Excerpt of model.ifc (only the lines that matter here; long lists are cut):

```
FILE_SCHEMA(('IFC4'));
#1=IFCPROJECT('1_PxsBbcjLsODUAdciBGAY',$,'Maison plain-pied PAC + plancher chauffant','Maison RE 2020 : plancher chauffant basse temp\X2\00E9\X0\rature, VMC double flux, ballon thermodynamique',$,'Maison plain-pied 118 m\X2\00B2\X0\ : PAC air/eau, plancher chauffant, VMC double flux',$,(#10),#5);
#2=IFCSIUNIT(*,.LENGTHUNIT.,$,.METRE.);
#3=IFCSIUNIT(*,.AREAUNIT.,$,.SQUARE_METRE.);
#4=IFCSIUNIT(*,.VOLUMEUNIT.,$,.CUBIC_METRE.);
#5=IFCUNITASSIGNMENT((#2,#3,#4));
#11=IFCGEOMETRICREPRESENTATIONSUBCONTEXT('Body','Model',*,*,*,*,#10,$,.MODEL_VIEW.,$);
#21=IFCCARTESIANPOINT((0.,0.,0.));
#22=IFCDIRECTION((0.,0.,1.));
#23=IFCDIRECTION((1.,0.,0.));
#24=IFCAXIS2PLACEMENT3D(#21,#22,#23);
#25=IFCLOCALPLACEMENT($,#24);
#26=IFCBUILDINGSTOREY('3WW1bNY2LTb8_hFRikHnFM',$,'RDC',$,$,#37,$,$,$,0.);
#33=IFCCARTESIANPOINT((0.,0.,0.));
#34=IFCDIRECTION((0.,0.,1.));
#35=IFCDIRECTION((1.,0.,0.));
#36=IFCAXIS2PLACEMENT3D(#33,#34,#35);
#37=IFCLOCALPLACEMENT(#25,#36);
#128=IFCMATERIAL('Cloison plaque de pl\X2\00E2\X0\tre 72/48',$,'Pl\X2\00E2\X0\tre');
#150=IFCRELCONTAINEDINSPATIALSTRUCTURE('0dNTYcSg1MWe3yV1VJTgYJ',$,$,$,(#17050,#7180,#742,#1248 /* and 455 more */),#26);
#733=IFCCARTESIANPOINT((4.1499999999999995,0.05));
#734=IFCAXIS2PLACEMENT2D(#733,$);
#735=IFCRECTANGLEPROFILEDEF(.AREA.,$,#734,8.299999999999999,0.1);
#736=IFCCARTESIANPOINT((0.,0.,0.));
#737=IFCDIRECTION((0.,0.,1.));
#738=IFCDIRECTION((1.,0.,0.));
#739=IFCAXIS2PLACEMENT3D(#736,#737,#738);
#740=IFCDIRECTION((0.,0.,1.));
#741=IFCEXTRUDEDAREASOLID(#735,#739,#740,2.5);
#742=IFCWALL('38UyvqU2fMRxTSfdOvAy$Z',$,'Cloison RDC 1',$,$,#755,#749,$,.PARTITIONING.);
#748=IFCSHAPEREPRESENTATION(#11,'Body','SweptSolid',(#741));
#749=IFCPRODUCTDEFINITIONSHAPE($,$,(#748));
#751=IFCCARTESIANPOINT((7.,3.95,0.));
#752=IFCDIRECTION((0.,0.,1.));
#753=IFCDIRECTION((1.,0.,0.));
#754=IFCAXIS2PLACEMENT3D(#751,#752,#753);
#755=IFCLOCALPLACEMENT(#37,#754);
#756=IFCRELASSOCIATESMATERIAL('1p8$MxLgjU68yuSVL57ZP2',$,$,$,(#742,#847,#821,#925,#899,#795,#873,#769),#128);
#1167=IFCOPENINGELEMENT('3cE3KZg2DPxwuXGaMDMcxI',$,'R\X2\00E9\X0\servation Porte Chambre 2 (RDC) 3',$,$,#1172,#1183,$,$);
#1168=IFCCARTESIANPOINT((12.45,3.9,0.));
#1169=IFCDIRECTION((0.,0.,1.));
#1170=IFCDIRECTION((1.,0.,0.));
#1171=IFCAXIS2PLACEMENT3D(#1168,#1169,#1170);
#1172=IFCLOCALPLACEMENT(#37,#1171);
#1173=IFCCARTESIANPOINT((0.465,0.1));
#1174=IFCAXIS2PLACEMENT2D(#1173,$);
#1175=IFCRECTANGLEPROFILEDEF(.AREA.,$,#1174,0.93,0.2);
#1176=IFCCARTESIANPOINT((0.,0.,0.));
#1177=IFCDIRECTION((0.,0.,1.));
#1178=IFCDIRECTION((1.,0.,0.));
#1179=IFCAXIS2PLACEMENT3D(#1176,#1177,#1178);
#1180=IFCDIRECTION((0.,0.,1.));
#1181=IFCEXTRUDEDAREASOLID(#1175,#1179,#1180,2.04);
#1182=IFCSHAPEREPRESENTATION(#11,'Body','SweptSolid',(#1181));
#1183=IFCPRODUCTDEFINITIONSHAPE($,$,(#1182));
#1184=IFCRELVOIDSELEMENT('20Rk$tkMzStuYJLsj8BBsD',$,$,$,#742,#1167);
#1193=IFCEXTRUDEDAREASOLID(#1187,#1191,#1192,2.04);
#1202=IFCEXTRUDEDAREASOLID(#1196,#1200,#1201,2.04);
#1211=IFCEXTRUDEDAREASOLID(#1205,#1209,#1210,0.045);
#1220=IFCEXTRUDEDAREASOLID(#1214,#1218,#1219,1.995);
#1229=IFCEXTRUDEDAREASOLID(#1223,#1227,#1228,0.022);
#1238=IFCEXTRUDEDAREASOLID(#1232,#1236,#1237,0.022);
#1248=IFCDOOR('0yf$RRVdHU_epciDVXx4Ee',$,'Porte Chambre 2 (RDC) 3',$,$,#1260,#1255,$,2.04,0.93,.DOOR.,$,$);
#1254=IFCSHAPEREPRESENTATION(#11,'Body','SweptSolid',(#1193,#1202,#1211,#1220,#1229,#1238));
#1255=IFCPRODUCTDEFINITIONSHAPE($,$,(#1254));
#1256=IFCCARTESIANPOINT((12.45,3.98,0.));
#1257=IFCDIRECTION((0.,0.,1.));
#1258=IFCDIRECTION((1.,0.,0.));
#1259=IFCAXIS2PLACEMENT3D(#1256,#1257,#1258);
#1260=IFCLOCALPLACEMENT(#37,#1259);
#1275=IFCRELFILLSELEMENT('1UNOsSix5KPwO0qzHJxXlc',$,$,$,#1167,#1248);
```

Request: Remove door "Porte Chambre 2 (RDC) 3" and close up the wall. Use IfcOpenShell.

```python
import ifcopenshell
import ifcopenshell.api.feature
import ifcopenshell.api.root
import ifcopenshell.geom
import ifcopenshell.util.shape

model = ifcopenshell.open("model.ifc")
settings = ifcopenshell.geom.settings()


def volume(element):
    """Net volume in cubic metres, openings subtracted."""
    shape = ifcopenshell.geom.create_shape(settings, element)
    return ifcopenshell.util.shape.get_volume(shape.geometry)


door = model.by_id(1248)
opening = door.FillsVoids[0].RelatingOpeningElement
wall = opening.VoidsElements[0].RelatingBuildingElement
before = volume(wall)

ifcopenshell.api.root.remove_product(model, product=door)
ifcopenshell.api.feature.remove_feature(model, feature=opening)

after = volume(wall)

print(f"wall volume {before:.3f} -> {after:.3f} m3")

model.write("model_v2.ifc")
```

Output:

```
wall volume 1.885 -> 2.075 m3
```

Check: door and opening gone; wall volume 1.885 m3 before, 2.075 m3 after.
